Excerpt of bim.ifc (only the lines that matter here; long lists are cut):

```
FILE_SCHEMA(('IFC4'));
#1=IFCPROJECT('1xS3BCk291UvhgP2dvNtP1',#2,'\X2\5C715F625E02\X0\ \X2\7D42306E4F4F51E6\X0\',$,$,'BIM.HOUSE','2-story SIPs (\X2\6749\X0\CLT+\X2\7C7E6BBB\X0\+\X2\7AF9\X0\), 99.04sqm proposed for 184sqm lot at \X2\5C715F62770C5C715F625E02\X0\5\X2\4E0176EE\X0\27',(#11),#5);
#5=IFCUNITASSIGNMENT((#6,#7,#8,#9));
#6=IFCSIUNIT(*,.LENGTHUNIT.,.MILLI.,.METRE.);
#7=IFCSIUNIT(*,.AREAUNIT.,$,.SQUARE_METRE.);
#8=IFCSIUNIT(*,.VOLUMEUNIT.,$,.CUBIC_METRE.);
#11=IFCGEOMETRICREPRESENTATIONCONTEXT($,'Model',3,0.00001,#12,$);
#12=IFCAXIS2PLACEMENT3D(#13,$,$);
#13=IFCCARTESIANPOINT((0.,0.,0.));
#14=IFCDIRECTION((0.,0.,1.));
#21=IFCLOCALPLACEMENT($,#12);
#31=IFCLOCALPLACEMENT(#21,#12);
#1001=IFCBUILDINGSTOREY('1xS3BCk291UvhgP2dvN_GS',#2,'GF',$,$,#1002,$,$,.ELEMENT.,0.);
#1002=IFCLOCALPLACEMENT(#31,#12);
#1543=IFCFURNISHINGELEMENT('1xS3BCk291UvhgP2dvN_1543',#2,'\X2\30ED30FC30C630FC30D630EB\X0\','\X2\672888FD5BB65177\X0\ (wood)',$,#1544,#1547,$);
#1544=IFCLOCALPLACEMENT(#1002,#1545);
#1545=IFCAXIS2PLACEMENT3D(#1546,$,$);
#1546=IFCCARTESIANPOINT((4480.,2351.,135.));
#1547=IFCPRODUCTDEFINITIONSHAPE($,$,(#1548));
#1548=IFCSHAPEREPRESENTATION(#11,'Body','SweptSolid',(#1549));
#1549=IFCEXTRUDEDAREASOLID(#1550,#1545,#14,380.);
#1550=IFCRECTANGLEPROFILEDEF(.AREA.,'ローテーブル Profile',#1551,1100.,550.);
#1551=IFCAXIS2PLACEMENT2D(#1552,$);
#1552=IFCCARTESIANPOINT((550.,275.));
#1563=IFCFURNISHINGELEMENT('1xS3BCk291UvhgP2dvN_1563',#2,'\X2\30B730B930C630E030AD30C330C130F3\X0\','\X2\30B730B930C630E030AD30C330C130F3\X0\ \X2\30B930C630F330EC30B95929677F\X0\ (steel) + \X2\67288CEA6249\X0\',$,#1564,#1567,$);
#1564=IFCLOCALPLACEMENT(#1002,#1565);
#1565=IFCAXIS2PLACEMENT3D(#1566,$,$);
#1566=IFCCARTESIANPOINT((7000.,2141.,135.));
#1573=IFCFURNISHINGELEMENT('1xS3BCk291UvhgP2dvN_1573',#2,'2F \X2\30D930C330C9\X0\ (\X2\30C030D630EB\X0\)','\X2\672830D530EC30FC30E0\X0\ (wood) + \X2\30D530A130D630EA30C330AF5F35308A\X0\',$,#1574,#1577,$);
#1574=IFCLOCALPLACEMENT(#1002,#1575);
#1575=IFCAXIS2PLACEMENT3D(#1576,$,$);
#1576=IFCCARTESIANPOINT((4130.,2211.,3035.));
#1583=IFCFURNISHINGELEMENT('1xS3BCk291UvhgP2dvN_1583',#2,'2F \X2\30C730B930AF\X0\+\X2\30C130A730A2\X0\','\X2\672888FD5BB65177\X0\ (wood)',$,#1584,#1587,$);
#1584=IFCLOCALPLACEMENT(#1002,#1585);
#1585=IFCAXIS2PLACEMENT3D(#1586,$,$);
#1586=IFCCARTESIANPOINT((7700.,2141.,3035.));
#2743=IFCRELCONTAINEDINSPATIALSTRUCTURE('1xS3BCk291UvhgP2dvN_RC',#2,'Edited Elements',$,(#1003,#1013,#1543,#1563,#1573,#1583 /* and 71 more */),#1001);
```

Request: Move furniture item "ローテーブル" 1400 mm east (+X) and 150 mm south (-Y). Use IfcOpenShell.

```python
import ifcopenshell
import ifcopenshell.api.geometry
import ifcopenshell.util.placement
import ifcopenshell.util.unit

model = ifcopenshell.open("bim.ifc")
unit_scale = ifcopenshell.util.unit.calculate_unit_scale(model)

item = model.by_guid("1xS3BCk291UvhgP2dvN_1543")
matrix = ifcopenshell.util.placement.get_local_placement(item.ObjectPlacement)
matrix[0, 3] += 1.4 / unit_scale
matrix[1, 3] -= 0.15 / unit_scale
ifcopenshell.api.geometry.edit_object_placement(model, product=item, matrix=matrix, is_si=False)

print(ifcopenshell.util.placement.get_local_placement(item.ObjectPlacement).round(3) + 0.0)

model.write("bim_updated.ifc")
```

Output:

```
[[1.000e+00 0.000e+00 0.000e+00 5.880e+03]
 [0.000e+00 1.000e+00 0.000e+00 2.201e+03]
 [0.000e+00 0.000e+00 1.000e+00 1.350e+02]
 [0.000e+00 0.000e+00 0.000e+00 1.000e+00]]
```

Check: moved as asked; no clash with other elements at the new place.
